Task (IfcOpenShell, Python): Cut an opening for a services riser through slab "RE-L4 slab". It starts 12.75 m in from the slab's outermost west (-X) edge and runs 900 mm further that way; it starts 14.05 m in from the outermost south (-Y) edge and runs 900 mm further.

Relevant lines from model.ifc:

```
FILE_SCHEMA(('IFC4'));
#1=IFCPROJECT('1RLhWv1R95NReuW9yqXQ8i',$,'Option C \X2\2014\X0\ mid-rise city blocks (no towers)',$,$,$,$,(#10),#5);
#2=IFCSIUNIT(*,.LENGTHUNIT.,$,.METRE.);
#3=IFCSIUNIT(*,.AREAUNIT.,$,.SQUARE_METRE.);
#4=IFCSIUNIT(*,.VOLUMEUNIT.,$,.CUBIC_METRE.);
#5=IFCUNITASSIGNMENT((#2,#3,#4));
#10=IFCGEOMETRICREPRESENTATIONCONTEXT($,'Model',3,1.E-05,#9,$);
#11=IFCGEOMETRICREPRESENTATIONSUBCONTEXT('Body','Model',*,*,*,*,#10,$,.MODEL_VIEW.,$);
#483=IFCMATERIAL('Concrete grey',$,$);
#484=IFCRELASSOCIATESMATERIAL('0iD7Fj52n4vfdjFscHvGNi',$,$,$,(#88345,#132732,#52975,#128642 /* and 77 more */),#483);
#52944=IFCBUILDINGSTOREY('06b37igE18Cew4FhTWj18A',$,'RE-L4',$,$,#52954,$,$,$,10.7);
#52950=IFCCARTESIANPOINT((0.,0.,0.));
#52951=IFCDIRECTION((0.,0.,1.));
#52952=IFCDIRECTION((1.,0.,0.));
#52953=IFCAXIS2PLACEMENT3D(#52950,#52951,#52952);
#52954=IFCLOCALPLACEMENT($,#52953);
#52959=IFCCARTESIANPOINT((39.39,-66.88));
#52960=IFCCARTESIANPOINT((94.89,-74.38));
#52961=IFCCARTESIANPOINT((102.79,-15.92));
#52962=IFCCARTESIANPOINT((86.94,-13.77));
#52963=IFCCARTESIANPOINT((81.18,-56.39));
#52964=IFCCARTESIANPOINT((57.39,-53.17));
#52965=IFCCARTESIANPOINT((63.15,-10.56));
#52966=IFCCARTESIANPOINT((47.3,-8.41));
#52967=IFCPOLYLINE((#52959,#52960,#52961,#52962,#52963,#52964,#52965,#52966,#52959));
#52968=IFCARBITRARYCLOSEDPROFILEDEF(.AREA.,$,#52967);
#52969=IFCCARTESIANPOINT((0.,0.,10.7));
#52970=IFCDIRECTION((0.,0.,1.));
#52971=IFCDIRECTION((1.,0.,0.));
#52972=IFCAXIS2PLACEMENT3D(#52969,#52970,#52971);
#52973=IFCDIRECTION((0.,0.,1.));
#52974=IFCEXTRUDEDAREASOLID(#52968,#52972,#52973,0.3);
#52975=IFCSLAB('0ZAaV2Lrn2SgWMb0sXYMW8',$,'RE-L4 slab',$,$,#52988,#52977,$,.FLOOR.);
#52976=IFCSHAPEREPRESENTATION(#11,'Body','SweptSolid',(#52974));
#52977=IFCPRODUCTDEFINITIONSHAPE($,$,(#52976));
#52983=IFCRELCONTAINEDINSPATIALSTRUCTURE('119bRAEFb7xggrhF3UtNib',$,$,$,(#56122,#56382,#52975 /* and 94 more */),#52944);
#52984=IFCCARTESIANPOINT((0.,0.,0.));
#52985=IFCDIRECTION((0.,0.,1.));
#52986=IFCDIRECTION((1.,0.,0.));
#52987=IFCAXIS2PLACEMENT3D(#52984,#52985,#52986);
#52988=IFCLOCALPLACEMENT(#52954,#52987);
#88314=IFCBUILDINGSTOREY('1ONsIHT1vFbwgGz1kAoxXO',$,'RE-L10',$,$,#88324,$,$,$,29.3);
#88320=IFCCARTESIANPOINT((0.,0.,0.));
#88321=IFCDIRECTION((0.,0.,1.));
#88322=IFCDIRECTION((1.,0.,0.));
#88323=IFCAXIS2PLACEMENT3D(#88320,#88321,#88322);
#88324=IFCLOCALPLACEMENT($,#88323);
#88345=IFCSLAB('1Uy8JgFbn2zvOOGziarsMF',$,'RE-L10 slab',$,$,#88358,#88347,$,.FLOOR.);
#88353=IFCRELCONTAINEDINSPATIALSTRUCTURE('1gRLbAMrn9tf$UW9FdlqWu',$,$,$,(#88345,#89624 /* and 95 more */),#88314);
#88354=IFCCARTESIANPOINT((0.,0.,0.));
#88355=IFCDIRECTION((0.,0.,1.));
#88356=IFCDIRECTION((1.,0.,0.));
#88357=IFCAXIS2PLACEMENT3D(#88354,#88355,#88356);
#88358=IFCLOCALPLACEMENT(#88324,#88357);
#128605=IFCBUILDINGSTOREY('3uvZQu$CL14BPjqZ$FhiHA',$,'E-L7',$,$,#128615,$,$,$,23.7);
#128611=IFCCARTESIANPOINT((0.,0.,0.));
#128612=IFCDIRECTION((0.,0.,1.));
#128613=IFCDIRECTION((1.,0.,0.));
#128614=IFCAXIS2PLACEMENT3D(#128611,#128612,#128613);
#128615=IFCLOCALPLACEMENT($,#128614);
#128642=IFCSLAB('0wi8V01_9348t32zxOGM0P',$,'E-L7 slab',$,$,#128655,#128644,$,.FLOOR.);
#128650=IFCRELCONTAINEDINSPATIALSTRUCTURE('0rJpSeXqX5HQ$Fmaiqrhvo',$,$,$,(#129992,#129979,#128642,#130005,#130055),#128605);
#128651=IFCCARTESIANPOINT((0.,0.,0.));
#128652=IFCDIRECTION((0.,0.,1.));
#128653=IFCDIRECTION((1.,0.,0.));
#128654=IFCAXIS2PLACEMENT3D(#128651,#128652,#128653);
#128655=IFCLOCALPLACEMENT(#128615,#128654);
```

```python
import numpy as np
import ifcopenshell
import ifcopenshell.api.feature
import ifcopenshell.api.geometry
import ifcopenshell.api.root
import ifcopenshell.geom
import ifcopenshell.util.placement
import ifcopenshell.util.representation
import ifcopenshell.util.shape
import ifcopenshell.util.unit

model = ifcopenshell.open("model.ifc")
unit_scale = ifcopenshell.util.unit.calculate_unit_scale(model)
settings = ifcopenshell.geom.settings()


def volume(element):
    """Net volume in cubic metres, openings subtracted."""
    shape = ifcopenshell.geom.create_shape(settings, element)
    return ifcopenshell.util.shape.get_volume(shape.geometry)


slab = model.by_guid("0ZAaV2Lrn2SgWMb0sXYMW8")
before = volume(slab)

# Extent in the slab's own axes, in metres. The edges named are its -X and -Y sides.
slab_shape = ifcopenshell.geom.create_shape(settings, slab)
vertices = ifcopenshell.util.shape.get_vertices(slab_shape.geometry)
x_min, y_min, bottom = vertices.min(axis=0)
top = vertices[:, 2].max()

opening = ifcopenshell.api.root.create_entity(model, ifc_class="IfcOpeningElement", name="Services riser opening", predefined_type="OPENING")
context = ifcopenshell.util.representation.get_context(model, "Model", "Body", "MODEL_VIEW")
width, depth = 0.9, 0.9
outline = [(0.0, 0.0), (width, 0.0), (width, depth), (0.0, depth), (0.0, 0.0)]
# Overshoot both faces by 50 mm so the cut is clean.
shape = ifcopenshell.api.geometry.add_slab_representation(
    model, context=context, depth=top - bottom + 0.1, polyline=outline
)
ifcopenshell.api.geometry.assign_representation(model, product=opening, representation=shape)

matrix = ifcopenshell.util.placement.get_local_placement(slab.ObjectPlacement)
matrix[:, 3] = matrix @ np.append(np.array([x_min + 12.75, y_min + 14.05, bottom - 0.05]) / unit_scale, 1.0)
ifcopenshell.api.geometry.edit_object_placement(model, product=opening, matrix=matrix, is_si=False)
ifcopenshell.api.feature.add_feature(model, feature=opening, element=slab)

after = volume(slab)

print(f"slab volume {before:.3f} -> {after:.3f} m3")

model.write("model_v2.ifc")
```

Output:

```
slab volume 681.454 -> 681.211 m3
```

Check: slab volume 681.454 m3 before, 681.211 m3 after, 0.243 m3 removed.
